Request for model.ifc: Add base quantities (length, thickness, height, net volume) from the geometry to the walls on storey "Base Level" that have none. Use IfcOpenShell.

First a look at what the model holds.

```python
import ifcopenshell
import ifcopenshell.util.element
import ifcopenshell.util.unit

model = ifcopenshell.open("model.ifc")
print(model.schema)
for unit_type in ("LENGTHUNIT", "AREAUNIT", "VOLUMEUNIT"):
    print(unit_type, ifcopenshell.util.unit.calculate_unit_scale(model, unit_type))
storey = next(s for s in model.by_type("IfcBuildingStorey") if s.Name == "Base Level")
walls = [e for e in ifcopenshell.util.element.get_decomposition(storey) if e.is_a("IfcWall")]
for e in sorted(walls, key=lambda e: e.id()):
    print(e.id(), e.is_a(), e.Name, list(ifcopenshell.util.element.get_psets(e, qtos_only=True)), sep=" | ")
```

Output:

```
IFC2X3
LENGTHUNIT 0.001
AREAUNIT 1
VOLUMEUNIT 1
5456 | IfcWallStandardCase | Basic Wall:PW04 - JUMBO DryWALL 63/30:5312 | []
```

```python
import ifcopenshell
import ifcopenshell.api.pset
import ifcopenshell.geom
import ifcopenshell.util.element
import ifcopenshell.util.shape
import ifcopenshell.util.unit

model = ifcopenshell.open("model.ifc")
unit_scale = ifcopenshell.util.unit.calculate_unit_scale(model)
volume_scale = ifcopenshell.util.unit.calculate_unit_scale(model, "VOLUMEUNIT")
settings = ifcopenshell.geom.settings()

storey = next(s for s in model.by_type("IfcBuildingStorey") if s.Name == "Base Level")
walls = [e for e in ifcopenshell.util.element.get_decomposition(storey) if e.is_a("IfcWall")]

for e in sorted(walls, key=lambda e: e.id()):
    if ifcopenshell.util.element.get_psets(e, qtos_only=True, should_inherit=False):
        continue
    # Geometry comes back in metres, in the element's own axes.
    shape = ifcopenshell.geom.create_shape(settings, e)
    values = {
        "Length": ifcopenshell.util.shape.get_x(shape.geometry) / unit_scale,
        "Width": ifcopenshell.util.shape.get_y(shape.geometry) / unit_scale,
        "Height": ifcopenshell.util.shape.get_z(shape.geometry) / unit_scale,
        "NetVolume": ifcopenshell.util.shape.get_volume(shape.geometry) / volume_scale,
    }
    qto = ifcopenshell.api.pset.add_qto(model, product=e, name="BaseQuantities")
    ifcopenshell.api.pset.edit_qto(model, qto=qto, properties=values)
    print(e.id(), {k: round(v, 3) for k, v in values.items()})

model.write("model_edited.ifc")
```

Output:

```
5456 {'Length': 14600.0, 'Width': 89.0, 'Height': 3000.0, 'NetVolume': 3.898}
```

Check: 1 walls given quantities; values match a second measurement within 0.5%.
